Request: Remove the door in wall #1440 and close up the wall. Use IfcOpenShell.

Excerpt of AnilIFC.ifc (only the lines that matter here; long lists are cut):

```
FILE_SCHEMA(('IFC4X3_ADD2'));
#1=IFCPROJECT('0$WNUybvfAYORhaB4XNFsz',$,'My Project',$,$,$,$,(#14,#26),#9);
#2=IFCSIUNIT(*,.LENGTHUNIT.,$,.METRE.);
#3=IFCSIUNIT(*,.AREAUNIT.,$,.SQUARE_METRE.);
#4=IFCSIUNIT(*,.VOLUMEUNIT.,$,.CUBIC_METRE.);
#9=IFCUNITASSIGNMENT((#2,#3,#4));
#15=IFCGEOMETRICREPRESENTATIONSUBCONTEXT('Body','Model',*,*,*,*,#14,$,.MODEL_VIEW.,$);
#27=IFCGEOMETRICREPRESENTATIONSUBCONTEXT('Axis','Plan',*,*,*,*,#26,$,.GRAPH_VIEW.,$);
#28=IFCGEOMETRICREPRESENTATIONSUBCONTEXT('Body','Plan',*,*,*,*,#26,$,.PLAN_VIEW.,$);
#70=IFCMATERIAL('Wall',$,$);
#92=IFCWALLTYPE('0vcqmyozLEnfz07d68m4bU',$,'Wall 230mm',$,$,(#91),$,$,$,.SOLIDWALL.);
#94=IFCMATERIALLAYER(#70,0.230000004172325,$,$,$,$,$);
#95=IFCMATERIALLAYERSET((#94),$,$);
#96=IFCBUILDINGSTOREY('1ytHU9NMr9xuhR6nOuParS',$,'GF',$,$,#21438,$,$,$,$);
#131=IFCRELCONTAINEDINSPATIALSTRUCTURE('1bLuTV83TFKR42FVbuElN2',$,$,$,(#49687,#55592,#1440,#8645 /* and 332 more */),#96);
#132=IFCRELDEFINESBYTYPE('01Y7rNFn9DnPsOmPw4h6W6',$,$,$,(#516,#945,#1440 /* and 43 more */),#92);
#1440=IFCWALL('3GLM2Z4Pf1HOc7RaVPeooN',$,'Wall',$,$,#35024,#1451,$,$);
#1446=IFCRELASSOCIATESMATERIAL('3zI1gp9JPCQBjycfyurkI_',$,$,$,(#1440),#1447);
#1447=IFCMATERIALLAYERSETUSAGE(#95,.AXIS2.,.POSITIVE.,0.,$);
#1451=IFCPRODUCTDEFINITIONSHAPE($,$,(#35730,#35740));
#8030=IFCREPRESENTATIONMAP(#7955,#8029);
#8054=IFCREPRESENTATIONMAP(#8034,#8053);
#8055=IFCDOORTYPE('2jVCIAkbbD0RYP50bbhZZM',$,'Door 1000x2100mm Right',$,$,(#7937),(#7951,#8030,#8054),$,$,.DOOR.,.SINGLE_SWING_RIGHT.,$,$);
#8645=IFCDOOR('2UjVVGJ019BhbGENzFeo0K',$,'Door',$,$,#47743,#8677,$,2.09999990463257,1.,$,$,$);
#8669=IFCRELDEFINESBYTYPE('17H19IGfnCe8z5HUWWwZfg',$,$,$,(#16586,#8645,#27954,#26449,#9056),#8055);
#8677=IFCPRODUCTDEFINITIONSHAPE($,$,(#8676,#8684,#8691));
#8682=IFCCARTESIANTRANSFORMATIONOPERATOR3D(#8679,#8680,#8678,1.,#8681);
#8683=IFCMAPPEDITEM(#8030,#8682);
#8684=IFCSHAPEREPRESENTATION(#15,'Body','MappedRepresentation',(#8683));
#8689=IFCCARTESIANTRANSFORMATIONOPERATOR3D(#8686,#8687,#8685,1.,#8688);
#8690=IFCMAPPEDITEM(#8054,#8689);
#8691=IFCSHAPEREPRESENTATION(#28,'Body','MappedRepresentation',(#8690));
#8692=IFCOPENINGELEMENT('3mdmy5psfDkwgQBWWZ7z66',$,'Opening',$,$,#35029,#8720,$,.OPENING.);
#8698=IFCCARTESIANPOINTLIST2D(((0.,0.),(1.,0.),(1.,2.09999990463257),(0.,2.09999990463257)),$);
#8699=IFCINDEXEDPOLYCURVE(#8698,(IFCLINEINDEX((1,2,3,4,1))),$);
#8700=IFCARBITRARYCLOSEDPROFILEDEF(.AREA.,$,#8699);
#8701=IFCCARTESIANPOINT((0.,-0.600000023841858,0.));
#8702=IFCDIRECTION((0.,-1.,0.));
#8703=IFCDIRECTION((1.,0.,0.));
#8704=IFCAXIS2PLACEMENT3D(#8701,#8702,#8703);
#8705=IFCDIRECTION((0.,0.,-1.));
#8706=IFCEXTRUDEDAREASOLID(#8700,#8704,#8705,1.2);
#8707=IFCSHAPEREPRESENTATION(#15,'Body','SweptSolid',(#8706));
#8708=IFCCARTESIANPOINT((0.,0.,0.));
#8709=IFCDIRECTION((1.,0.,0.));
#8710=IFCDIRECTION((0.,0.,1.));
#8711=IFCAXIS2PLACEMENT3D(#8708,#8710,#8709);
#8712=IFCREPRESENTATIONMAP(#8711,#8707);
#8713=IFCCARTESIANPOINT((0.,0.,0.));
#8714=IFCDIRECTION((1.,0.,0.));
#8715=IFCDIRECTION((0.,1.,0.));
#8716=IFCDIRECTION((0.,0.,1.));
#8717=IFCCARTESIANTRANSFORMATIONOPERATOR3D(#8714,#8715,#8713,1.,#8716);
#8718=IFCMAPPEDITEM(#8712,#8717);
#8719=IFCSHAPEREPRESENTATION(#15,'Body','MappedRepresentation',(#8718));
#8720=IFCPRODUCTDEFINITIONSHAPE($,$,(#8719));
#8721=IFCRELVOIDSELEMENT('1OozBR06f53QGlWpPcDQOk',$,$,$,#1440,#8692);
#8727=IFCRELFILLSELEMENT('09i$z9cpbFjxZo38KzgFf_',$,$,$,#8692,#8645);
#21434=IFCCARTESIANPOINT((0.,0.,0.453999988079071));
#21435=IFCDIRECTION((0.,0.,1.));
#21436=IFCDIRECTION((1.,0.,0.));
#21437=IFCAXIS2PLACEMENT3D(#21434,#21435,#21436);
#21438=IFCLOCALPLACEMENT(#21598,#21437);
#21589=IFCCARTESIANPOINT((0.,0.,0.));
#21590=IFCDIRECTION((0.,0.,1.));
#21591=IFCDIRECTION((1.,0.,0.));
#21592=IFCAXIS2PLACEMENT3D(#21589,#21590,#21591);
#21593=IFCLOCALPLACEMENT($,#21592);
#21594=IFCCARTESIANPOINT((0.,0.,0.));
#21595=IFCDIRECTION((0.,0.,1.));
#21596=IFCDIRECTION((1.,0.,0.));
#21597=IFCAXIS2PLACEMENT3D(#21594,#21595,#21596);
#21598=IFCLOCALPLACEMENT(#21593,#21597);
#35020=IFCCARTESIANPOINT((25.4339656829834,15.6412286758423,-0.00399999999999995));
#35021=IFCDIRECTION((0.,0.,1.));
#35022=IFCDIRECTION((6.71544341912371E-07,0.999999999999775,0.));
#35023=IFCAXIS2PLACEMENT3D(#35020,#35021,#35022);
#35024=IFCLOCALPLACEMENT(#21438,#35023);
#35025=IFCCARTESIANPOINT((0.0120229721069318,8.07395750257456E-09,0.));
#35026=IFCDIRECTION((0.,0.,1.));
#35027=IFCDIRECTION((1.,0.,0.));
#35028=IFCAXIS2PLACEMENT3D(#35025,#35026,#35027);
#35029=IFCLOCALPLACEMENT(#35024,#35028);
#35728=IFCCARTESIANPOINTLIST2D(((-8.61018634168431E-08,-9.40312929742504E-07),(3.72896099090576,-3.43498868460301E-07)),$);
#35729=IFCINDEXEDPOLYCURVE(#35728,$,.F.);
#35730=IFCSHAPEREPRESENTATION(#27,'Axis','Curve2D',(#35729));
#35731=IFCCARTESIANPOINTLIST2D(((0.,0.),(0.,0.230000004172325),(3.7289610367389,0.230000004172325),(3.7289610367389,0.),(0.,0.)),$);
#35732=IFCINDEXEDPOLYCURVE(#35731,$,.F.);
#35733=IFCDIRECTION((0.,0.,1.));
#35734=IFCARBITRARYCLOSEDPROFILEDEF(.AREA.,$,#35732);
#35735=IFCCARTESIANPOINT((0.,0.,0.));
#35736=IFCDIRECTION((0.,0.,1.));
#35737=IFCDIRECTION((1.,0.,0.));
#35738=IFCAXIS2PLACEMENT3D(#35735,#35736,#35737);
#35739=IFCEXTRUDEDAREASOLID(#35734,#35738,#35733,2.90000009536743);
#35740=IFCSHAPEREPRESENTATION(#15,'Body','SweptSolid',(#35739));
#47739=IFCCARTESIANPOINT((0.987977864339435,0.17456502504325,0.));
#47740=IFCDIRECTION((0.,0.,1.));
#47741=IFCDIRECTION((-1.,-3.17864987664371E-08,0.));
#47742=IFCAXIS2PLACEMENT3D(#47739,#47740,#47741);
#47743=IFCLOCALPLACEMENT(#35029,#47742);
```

```python
import ifcopenshell
import ifcopenshell.api.feature
import ifcopenshell.api.root
import ifcopenshell.geom
import ifcopenshell.util.shape

model = ifcopenshell.open("AnilIFC.ifc")
settings = ifcopenshell.geom.settings()


def volume(element):
    """Net volume in cubic metres, openings subtracted."""
    shape = ifcopenshell.geom.create_shape(settings, element)
    return ifcopenshell.util.shape.get_volume(shape.geometry)


door = model.by_guid("2UjVVGJ019BhbGENzFeo0K")
opening = door.FillsVoids[0].RelatingOpeningElement
wall = opening.VoidsElements[0].RelatingBuildingElement
before = volume(wall)

ifcopenshell.api.root.remove_product(model, product=door)
ifcopenshell.api.feature.remove_feature(model, feature=opening)

after = volume(wall)

print(f"wall volume {before:.3f} -> {after:.3f} m3")

model.write("AnilIFC-out.ifc")
```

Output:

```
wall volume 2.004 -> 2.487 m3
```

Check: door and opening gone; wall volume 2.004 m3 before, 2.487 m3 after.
